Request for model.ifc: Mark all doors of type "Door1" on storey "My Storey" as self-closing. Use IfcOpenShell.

First a look at what the model holds.

```python
import ifcopenshell
import ifcopenshell.util.element

model = ifcopenshell.open("model.ifc")
print(model.schema)
storey = next(s for s in model.by_type("IfcBuildingStorey") if s.Name == "My Storey")
doors = [e for e in ifcopenshell.util.element.get_decomposition(storey) if e.is_a("IfcDoor")]
seen = {}
for e in doors:
    element_type = ifcopenshell.util.element.get_type(e)
    key = (element_type.Name if element_type != e and element_type else None, ifcopenshell.util.element.get_pset(e, "Pset_DoorCommon", "SelfClosing"))
    seen[key] = seen.get(key, 0) + 1
for (name, value), count in sorted(seen.items(), key=str):
    print(count, "x", name, "|", value)
```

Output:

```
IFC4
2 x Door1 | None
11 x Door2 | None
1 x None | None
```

```python
import ifcopenshell
import ifcopenshell.api.pset
import ifcopenshell.util.element

model = ifcopenshell.open("model.ifc")

storey = next(s for s in model.by_type("IfcBuildingStorey") if s.Name == "My Storey")
doors = [e for e in ifcopenshell.util.element.get_decomposition(storey) if e.is_a("IfcDoor")]

count = 0
for e in doors:
    element_type = ifcopenshell.util.element.get_type(e)
    if element_type in (None, e) or element_type.Name != "Door1":
        continue
    # add_pset returns the element's existing set when there is one.
    pset = ifcopenshell.api.pset.add_pset(model, product=e, name="Pset_DoorCommon")
    ifcopenshell.api.pset.edit_pset(model, pset=pset, properties={"SelfClosing": True})
    count += 1

print(count, "doors updated")

model.write("model_v2.ifc")
```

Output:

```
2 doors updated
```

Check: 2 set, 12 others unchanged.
